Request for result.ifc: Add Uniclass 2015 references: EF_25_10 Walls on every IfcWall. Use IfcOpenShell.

First a look at what the model holds.

```python
import ifcopenshell

model = ifcopenshell.open("result.ifc")
print(model.schema)
print("classifications:", [c.Name for c in model.by_type("IfcClassification")])
for ifc_class in ("IfcDoor", "IfcRoof", "IfcStair", "IfcWall", "IfcWindow"):
    print(ifc_class, len(model.by_type(ifc_class)))
```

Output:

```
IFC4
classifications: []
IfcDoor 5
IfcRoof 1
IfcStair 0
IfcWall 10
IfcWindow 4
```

```python
import ifcopenshell
import ifcopenshell.api.classification

model = ifcopenshell.open("result.ifc")

system = ifcopenshell.api.classification.add_classification(model, classification="Uniclass 2015")

codes = {
    "IfcWall": ("EF_25_10", "Walls"),
}
for ifc_class, (code, name) in codes.items():
    products = model.by_type(ifc_class)
    ifcopenshell.api.classification.add_reference(
        model, products=products, classification=system, identification=code, name=name
    )
    print(code, len(products))

model.write("result_rev.ifc")
```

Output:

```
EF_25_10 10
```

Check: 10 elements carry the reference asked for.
